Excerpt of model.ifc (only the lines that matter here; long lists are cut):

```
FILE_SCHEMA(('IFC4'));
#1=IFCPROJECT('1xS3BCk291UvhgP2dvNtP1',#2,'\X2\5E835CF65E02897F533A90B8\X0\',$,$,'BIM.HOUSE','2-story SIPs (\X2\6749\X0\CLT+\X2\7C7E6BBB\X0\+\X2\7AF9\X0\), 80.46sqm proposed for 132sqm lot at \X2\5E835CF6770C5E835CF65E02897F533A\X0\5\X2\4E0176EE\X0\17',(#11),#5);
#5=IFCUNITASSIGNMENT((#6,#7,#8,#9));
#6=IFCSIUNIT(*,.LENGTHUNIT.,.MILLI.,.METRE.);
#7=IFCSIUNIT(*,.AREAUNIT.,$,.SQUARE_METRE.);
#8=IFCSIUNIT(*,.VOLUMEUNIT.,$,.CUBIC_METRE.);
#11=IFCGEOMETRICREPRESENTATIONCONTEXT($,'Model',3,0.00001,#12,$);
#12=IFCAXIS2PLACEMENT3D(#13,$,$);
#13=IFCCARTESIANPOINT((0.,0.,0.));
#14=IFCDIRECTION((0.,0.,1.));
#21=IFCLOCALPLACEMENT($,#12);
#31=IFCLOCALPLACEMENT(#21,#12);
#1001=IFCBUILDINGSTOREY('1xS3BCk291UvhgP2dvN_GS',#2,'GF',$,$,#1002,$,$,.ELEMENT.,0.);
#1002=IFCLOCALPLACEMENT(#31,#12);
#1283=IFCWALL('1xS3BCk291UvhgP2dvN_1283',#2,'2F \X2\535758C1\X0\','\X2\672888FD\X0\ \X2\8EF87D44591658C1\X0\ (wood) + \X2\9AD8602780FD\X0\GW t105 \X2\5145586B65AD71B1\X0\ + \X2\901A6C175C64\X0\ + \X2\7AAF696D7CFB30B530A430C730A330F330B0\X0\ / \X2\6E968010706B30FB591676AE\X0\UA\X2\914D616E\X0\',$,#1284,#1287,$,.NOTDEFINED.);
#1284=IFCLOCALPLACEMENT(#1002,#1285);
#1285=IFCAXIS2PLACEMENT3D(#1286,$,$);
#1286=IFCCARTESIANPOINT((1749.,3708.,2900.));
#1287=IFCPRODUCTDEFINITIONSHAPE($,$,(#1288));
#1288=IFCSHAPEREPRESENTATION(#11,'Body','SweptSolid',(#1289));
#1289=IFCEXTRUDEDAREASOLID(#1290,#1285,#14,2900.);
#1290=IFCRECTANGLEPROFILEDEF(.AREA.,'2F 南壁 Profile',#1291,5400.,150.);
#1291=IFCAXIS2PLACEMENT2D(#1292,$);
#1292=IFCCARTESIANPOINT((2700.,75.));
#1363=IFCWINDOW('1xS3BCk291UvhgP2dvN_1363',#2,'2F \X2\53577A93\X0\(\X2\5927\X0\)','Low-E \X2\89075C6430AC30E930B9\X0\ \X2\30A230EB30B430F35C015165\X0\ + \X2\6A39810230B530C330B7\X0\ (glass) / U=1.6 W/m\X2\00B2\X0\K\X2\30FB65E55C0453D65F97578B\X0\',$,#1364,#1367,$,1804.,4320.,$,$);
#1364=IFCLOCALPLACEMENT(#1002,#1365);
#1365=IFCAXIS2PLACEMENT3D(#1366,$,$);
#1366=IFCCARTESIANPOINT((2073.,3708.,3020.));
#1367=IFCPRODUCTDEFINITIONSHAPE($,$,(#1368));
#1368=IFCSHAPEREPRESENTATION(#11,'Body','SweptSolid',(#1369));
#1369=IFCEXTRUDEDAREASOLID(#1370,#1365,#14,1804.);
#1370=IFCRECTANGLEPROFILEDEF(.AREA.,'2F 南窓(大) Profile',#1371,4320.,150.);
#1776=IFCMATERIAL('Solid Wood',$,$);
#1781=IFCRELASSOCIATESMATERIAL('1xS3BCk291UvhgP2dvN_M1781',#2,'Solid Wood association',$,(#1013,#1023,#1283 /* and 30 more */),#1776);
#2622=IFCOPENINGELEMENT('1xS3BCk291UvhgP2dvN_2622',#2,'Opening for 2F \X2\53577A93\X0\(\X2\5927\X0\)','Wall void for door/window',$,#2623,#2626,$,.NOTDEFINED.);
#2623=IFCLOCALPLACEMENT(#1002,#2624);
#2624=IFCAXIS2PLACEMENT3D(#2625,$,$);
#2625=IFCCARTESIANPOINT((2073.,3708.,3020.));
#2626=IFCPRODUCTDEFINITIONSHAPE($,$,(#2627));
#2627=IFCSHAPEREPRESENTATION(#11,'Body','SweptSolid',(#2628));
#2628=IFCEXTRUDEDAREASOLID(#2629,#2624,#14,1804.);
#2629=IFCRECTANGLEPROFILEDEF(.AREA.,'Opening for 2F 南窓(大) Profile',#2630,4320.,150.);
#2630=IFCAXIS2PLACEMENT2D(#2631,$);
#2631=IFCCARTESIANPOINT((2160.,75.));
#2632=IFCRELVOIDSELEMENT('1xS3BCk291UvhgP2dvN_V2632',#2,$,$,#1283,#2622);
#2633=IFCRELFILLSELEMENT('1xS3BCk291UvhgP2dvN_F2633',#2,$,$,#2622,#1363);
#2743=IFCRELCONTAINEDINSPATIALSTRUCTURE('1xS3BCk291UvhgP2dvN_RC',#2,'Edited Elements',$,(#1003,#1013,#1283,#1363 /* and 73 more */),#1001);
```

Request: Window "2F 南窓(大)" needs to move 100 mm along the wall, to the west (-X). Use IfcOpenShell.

```python
import ifcopenshell
import ifcopenshell.api.geometry
import ifcopenshell.util.placement
import ifcopenshell.util.unit

model = ifcopenshell.open("model.ifc")
unit_scale = ifcopenshell.util.unit.calculate_unit_scale(model)

window = model.by_guid("1xS3BCk291UvhgP2dvN_1363")
opening = window.FillsVoids[0].RelatingOpeningElement
wall = opening.VoidsElements[0].RelatingBuildingElement

wall_matrix = ifcopenshell.util.placement.get_local_placement(wall.ObjectPlacement)
shift = wall_matrix[:3, 0] * -0.1 / unit_scale
before = ifcopenshell.util.placement.get_local_placement(window.ObjectPlacement)[:3, 3].copy()

# The window is not placed relative to its opening, so move both.
for product in (opening, window):
    matrix = ifcopenshell.util.placement.get_local_placement(product.ObjectPlacement)
    matrix[:3, 3] += shift
    ifcopenshell.api.geometry.edit_object_placement(model, product=product, matrix=matrix, is_si=False)

after = ifcopenshell.util.placement.get_local_placement(window.ObjectPlacement)[:3, 3]
print("window moved by", (after - before).round(3) + 0.0)

model.write("model_v2.ifc")
```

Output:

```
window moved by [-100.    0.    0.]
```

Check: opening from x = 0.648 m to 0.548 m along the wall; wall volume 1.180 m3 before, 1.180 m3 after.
